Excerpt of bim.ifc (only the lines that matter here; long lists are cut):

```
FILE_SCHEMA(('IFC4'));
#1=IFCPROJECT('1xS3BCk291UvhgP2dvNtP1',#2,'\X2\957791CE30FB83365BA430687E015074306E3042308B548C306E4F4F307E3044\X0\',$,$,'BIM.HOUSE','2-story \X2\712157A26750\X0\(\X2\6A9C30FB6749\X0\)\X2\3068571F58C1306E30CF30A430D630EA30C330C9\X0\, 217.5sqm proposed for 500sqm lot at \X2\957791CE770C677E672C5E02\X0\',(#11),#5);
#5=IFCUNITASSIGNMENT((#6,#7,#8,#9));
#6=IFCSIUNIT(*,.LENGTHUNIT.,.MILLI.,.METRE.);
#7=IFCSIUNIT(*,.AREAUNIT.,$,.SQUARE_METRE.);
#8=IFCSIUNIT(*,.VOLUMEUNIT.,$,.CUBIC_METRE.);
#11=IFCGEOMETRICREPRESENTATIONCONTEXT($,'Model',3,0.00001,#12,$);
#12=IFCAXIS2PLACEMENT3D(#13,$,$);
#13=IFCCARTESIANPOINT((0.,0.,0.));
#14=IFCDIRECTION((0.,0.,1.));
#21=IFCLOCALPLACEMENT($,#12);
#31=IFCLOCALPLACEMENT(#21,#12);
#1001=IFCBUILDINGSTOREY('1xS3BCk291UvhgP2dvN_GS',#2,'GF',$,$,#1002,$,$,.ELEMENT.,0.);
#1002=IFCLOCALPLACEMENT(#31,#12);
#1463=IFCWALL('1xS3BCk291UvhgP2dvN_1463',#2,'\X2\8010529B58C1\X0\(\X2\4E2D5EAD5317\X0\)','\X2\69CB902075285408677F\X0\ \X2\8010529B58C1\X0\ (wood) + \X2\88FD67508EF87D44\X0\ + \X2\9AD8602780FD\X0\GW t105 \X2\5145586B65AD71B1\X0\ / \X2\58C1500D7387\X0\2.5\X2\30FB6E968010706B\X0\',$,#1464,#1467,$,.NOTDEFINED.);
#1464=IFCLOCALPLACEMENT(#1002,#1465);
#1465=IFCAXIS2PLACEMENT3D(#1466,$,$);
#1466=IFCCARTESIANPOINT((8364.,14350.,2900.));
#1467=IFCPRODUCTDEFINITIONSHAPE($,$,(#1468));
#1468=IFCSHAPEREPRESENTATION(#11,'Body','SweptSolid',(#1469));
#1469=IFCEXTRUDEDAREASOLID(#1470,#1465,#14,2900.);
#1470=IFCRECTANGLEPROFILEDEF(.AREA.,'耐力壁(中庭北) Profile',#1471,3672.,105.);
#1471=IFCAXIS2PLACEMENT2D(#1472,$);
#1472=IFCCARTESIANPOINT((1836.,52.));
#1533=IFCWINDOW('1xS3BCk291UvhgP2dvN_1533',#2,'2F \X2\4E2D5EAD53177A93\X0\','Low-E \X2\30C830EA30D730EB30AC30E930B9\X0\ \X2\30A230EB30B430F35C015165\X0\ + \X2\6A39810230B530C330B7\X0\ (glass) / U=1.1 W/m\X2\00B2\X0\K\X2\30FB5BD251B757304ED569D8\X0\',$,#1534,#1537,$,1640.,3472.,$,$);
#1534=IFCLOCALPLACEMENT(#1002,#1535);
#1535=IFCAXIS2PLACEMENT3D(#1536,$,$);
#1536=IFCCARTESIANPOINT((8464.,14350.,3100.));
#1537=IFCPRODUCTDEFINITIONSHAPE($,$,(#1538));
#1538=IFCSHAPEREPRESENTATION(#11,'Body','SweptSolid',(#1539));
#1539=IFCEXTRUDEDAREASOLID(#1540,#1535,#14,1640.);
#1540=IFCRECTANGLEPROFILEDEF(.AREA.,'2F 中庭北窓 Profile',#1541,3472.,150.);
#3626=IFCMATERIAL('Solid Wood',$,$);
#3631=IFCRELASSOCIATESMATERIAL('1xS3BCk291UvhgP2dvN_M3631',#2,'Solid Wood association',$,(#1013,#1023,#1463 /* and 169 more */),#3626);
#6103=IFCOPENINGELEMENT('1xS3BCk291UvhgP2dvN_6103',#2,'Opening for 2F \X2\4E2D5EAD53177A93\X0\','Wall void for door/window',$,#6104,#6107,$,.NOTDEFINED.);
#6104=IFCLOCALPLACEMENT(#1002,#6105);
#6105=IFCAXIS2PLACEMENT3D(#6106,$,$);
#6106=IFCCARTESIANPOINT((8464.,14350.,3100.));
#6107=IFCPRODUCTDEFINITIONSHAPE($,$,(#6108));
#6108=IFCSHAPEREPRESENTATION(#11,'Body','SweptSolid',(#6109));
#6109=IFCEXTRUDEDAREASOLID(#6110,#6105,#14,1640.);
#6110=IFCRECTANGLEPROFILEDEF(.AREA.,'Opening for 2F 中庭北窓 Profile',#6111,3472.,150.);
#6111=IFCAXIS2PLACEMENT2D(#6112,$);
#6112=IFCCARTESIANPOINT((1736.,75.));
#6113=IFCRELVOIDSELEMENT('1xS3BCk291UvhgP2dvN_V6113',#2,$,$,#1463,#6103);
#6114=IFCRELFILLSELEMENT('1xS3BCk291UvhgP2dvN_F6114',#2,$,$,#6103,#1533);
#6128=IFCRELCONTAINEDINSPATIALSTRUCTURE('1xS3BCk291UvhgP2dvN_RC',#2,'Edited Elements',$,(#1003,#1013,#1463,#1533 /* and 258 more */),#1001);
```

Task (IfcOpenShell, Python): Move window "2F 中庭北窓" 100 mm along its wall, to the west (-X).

```python
import ifcopenshell
import ifcopenshell.api.geometry
import ifcopenshell.util.placement
import ifcopenshell.util.unit

model = ifcopenshell.open("bim.ifc")
unit_scale = ifcopenshell.util.unit.calculate_unit_scale(model)

window = model.by_guid("1xS3BCk291UvhgP2dvN_1533")
opening = window.FillsVoids[0].RelatingOpeningElement
wall = opening.VoidsElements[0].RelatingBuildingElement

wall_matrix = ifcopenshell.util.placement.get_local_placement(wall.ObjectPlacement)
shift = wall_matrix[:3, 0] * -0.1 / unit_scale
before = ifcopenshell.util.placement.get_local_placement(window.ObjectPlacement)[:3, 3].copy()

# The window is not placed relative to its opening, so move both.
for product in (opening, window):
    matrix = ifcopenshell.util.placement.get_local_placement(product.ObjectPlacement)
    matrix[:3, 3] += shift
    ifcopenshell.api.geometry.edit_object_placement(model, product=product, matrix=matrix, is_si=False)

after = ifcopenshell.util.placement.get_local_placement(window.ObjectPlacement)[:3, 3]
print("window moved by", (after - before).round(3) + 0.0)

model.write("bim_updated.ifc")
```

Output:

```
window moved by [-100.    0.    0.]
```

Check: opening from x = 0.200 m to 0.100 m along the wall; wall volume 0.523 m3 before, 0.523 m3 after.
